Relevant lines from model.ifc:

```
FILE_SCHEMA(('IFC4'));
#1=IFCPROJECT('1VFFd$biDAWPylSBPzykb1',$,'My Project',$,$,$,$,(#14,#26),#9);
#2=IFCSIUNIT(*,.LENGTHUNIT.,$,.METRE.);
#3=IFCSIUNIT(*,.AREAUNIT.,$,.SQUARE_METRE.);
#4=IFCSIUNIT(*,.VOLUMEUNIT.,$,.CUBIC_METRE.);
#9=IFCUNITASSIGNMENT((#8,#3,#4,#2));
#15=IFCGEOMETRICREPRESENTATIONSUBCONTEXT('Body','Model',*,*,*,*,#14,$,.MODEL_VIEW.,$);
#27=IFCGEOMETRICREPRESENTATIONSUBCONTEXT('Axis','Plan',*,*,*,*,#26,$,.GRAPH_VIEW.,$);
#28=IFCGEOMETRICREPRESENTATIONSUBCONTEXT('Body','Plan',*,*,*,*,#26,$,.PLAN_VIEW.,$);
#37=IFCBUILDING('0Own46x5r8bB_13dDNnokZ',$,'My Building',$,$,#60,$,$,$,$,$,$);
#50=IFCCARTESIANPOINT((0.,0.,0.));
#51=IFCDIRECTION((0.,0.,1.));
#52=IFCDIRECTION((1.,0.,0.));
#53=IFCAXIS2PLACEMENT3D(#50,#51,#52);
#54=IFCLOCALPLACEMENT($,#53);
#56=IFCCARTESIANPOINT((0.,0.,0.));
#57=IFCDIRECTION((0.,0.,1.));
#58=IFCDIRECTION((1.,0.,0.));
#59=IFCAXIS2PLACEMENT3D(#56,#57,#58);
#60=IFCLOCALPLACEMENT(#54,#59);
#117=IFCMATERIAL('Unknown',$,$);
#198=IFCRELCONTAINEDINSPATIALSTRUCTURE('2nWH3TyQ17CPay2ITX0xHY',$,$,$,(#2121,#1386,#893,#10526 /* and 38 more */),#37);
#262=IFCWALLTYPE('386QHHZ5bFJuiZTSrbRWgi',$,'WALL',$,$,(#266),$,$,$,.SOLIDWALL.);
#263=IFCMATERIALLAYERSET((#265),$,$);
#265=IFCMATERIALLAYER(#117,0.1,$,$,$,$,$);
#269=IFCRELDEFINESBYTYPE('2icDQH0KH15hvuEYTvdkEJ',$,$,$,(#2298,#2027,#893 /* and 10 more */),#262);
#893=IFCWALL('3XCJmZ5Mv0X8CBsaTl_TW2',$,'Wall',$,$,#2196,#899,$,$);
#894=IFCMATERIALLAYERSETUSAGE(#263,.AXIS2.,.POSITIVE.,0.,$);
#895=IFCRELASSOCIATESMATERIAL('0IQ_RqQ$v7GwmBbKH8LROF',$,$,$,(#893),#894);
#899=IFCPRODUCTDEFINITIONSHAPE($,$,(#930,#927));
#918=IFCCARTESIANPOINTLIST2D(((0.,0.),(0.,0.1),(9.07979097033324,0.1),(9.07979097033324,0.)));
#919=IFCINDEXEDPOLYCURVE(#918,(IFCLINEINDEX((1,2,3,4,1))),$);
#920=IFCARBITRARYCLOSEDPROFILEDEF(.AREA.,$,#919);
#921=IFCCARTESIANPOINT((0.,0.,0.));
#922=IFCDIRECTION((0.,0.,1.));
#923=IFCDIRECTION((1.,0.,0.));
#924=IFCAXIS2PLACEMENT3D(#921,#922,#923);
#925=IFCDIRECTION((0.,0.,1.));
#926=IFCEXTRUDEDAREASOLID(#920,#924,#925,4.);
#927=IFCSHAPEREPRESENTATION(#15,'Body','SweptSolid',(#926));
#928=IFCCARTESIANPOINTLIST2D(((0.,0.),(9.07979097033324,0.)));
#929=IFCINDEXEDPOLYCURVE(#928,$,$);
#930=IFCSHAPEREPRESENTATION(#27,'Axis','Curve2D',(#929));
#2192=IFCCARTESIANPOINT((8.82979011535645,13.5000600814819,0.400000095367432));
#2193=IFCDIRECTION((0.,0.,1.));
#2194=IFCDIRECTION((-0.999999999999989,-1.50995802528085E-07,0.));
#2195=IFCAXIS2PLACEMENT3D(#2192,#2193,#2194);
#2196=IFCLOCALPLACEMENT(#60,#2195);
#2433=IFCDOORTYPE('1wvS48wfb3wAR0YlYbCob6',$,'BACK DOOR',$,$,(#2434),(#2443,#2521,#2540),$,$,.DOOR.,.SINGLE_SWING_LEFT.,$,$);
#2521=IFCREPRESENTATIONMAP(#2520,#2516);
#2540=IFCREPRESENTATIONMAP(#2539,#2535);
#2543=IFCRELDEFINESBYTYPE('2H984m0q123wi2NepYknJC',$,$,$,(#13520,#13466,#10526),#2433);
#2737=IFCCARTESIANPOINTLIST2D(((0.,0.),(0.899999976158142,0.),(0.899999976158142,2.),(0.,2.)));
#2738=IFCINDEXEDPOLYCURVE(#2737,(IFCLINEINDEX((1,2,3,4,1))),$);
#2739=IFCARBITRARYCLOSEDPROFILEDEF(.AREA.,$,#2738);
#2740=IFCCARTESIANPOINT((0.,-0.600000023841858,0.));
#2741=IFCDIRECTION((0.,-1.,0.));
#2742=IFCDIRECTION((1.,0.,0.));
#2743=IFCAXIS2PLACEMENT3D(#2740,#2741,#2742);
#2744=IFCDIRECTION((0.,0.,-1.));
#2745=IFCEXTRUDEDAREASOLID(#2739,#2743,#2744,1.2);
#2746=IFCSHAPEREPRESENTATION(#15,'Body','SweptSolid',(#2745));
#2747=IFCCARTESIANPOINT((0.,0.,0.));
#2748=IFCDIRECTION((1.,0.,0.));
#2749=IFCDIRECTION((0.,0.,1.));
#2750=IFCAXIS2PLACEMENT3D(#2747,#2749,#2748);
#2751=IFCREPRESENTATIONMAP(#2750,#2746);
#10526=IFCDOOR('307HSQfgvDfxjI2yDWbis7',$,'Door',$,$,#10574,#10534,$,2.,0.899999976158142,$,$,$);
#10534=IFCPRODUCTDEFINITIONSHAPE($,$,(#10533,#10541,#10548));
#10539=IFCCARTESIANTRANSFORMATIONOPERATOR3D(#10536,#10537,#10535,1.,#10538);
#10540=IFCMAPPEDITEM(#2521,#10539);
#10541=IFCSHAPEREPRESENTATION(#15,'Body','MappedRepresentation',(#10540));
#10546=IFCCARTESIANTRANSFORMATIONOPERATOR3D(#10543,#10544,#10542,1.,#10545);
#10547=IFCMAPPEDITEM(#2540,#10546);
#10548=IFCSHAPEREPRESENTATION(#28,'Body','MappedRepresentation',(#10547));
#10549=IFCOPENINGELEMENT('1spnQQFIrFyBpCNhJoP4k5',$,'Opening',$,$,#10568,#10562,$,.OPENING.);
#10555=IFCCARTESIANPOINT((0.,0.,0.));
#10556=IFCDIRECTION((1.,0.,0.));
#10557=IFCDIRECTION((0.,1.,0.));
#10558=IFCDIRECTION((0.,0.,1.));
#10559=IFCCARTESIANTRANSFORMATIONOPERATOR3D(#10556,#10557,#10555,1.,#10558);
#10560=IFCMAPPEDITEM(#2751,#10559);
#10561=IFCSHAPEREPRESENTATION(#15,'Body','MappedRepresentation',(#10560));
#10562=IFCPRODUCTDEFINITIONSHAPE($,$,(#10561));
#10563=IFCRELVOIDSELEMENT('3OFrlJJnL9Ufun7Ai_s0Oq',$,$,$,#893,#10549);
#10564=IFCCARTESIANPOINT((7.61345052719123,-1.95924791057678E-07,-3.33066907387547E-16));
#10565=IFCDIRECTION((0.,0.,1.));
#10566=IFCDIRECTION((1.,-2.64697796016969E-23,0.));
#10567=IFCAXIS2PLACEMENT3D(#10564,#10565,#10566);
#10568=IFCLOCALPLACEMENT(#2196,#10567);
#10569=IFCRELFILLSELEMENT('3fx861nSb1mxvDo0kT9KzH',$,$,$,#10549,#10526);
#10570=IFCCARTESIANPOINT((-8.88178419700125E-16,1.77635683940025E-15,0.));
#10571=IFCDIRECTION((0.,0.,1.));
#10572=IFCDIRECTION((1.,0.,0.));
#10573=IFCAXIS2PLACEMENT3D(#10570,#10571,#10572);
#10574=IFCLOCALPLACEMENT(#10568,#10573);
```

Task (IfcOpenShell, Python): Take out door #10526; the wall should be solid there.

```python
import ifcopenshell
import ifcopenshell.api.feature
import ifcopenshell.api.root
import ifcopenshell.geom
import ifcopenshell.util.shape

model = ifcopenshell.open("model.ifc")
settings = ifcopenshell.geom.settings()


def volume(element):
    """Net volume in cubic metres, openings subtracted."""
    shape = ifcopenshell.geom.create_shape(settings, element)
    return ifcopenshell.util.shape.get_volume(shape.geometry)


door = model.by_guid("307HSQfgvDfxjI2yDWbis7")
opening = door.FillsVoids[0].RelatingOpeningElement
wall = opening.VoidsElements[0].RelatingBuildingElement
before = volume(wall)

ifcopenshell.api.root.remove_product(model, product=door)
ifcopenshell.api.feature.remove_feature(model, feature=opening)

after = volume(wall)

print(f"wall volume {before:.3f} -> {after:.3f} m3")

model.write("model-out.ifc")
```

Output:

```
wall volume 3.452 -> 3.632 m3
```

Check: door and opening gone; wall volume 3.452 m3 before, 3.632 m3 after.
